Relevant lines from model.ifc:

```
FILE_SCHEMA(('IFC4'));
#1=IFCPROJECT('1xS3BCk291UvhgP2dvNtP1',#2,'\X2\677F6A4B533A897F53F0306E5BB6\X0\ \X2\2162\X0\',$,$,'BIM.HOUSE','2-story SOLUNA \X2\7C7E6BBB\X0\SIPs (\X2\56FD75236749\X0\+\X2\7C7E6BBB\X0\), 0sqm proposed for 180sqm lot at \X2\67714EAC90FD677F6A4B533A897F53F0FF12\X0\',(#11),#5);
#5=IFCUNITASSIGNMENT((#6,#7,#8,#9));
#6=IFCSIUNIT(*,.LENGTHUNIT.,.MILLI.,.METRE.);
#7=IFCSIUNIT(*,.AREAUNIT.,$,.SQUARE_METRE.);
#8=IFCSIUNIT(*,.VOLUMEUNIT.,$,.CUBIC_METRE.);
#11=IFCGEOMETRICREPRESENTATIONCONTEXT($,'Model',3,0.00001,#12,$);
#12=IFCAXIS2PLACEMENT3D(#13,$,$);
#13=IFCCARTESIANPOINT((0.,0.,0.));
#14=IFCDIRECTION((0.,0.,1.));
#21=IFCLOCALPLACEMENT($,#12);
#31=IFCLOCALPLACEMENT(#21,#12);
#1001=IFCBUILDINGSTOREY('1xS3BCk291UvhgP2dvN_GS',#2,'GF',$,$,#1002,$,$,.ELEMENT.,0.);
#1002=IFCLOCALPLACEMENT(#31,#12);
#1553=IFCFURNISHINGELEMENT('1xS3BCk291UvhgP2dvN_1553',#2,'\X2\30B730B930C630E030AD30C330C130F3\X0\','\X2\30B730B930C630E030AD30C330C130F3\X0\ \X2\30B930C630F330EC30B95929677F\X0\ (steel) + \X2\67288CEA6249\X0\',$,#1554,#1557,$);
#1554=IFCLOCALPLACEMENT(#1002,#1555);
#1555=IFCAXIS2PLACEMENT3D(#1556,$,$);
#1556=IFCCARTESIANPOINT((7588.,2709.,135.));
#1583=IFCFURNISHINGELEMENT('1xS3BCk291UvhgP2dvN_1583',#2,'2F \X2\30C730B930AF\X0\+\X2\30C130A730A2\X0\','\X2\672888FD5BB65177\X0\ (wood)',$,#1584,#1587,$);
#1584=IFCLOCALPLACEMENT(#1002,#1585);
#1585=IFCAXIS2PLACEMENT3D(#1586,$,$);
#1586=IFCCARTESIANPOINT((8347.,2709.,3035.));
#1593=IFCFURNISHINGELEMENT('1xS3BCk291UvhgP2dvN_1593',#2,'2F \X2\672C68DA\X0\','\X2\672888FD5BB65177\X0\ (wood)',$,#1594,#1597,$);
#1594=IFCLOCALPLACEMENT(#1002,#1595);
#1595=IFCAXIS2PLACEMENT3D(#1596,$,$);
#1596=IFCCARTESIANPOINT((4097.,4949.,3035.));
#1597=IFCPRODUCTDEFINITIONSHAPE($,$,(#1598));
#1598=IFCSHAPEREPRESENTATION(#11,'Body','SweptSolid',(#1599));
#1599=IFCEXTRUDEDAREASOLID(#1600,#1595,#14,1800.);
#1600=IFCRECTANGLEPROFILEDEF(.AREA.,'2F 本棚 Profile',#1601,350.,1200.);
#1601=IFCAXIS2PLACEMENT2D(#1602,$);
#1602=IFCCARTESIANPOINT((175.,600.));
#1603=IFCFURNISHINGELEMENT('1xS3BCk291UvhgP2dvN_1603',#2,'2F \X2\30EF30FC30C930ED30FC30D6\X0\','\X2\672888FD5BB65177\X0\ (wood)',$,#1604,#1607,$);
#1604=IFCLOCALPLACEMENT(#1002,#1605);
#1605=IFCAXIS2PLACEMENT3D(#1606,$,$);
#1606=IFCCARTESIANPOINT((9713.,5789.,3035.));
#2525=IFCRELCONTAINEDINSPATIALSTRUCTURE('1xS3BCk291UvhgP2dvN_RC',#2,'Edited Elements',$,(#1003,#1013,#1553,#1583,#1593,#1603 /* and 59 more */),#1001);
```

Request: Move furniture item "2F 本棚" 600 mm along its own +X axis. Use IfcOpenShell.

```python
import ifcopenshell
import ifcopenshell.api.geometry
import ifcopenshell.util.placement

model = ifcopenshell.open("model.ifc")

item = model.by_guid("1xS3BCk291UvhgP2dvN_1593")
matrix = ifcopenshell.util.placement.get_local_placement(item.ObjectPlacement)
matrix[:3, 3] += matrix[:3, 0] * 600.0
ifcopenshell.api.geometry.edit_object_placement(model, product=item, matrix=matrix, is_si=False)

print(ifcopenshell.util.placement.get_local_placement(item.ObjectPlacement).round(3) + 0.0)

model.write("model_edited.ifc")
```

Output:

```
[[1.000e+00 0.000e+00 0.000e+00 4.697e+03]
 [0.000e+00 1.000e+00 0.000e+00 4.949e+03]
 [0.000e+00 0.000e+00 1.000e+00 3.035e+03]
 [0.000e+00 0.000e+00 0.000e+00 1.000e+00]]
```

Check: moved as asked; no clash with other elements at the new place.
